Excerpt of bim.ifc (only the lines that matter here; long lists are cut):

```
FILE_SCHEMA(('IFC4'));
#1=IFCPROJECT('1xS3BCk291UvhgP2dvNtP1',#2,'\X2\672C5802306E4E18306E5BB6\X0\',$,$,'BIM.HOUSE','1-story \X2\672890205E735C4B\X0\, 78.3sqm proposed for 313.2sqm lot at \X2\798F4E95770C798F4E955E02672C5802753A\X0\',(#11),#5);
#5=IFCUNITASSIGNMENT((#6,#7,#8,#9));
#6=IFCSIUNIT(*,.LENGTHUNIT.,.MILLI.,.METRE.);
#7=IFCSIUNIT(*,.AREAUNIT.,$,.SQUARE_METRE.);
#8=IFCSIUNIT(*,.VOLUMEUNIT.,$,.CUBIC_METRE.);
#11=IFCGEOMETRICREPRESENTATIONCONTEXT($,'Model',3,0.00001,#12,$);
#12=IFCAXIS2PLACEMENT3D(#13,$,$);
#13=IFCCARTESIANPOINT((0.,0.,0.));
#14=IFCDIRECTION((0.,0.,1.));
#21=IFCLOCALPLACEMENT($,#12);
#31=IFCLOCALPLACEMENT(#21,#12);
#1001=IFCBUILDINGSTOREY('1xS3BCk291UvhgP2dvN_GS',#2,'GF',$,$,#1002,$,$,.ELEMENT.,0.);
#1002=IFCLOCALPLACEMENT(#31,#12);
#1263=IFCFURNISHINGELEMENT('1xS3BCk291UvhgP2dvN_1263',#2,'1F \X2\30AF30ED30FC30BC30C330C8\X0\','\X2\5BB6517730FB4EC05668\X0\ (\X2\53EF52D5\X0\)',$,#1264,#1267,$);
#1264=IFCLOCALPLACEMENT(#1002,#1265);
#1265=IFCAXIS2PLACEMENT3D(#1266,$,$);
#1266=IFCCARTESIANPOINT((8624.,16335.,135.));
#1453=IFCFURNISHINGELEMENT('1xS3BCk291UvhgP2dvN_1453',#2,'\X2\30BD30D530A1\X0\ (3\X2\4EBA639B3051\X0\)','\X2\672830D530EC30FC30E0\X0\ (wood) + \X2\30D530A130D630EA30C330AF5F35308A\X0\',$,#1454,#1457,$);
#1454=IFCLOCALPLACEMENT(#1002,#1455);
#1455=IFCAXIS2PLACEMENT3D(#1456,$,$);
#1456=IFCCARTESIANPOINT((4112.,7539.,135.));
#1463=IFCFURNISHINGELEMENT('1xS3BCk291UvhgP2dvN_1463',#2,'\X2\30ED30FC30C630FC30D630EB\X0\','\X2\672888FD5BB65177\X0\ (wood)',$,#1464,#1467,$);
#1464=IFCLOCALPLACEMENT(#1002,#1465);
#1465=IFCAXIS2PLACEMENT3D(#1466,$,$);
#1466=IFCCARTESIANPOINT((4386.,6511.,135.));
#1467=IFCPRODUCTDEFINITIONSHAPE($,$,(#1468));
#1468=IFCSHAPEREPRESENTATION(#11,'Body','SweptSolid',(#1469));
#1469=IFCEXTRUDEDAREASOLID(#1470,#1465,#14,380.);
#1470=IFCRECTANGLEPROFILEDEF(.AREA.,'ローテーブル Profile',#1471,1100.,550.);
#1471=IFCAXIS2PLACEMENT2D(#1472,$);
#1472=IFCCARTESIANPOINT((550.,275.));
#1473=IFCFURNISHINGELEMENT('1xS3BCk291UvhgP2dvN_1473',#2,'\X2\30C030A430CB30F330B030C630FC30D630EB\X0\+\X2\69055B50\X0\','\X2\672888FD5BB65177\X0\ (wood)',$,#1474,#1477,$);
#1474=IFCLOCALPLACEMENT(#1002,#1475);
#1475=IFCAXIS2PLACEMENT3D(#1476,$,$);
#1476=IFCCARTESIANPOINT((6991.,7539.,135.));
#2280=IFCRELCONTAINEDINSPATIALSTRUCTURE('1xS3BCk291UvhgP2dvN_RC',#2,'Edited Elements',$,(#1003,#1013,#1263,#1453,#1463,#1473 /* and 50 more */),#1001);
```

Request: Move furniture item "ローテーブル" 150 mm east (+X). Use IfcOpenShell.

```python
import ifcopenshell
import ifcopenshell.api.geometry
import ifcopenshell.util.placement

model = ifcopenshell.open("bim.ifc")

item = model.by_id(1463)
matrix = ifcopenshell.util.placement.get_local_placement(item.ObjectPlacement)
matrix[0, 3] += 150.0
ifcopenshell.api.geometry.edit_object_placement(model, product=item, matrix=matrix, is_si=False)

print(ifcopenshell.util.placement.get_local_placement(item.ObjectPlacement).round(3) + 0.0)

model.write("bim_updated.ifc")
```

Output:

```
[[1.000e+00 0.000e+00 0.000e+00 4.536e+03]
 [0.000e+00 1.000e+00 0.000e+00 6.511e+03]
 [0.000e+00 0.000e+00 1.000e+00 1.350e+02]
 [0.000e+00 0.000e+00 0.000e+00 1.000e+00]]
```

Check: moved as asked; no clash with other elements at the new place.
